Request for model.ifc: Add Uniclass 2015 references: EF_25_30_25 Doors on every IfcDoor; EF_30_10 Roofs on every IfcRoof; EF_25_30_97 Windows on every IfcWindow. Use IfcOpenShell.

First a look at what the model holds.

```python
import ifcopenshell

model = ifcopenshell.open("model.ifc")
print(model.schema)
print("classifications:", [c.Name for c in model.by_type("IfcClassification")])
for ifc_class in ("IfcDoor", "IfcRoof", "IfcStair", "IfcWall", "IfcWindow"):
    print(ifc_class, len(model.by_type(ifc_class)))
```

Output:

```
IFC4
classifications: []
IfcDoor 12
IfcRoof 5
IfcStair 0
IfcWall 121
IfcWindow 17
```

```python
import ifcopenshell
import ifcopenshell.api.classification

model = ifcopenshell.open("model.ifc")

system = ifcopenshell.api.classification.add_classification(model, classification="Uniclass 2015")

codes = {
    "IfcDoor": ("EF_25_30_25", "Doors"),
    "IfcRoof": ("EF_30_10", "Roofs"),
    "IfcWindow": ("EF_25_30_97", "Windows"),
}
for ifc_class, (code, name) in codes.items():
    products = model.by_type(ifc_class)
    ifcopenshell.api.classification.add_reference(
        model, products=products, classification=system, identification=code, name=name
    )
    print(code, len(products))

model.write("model_v2.ifc")
```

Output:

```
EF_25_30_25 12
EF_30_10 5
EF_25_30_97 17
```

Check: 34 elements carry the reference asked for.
